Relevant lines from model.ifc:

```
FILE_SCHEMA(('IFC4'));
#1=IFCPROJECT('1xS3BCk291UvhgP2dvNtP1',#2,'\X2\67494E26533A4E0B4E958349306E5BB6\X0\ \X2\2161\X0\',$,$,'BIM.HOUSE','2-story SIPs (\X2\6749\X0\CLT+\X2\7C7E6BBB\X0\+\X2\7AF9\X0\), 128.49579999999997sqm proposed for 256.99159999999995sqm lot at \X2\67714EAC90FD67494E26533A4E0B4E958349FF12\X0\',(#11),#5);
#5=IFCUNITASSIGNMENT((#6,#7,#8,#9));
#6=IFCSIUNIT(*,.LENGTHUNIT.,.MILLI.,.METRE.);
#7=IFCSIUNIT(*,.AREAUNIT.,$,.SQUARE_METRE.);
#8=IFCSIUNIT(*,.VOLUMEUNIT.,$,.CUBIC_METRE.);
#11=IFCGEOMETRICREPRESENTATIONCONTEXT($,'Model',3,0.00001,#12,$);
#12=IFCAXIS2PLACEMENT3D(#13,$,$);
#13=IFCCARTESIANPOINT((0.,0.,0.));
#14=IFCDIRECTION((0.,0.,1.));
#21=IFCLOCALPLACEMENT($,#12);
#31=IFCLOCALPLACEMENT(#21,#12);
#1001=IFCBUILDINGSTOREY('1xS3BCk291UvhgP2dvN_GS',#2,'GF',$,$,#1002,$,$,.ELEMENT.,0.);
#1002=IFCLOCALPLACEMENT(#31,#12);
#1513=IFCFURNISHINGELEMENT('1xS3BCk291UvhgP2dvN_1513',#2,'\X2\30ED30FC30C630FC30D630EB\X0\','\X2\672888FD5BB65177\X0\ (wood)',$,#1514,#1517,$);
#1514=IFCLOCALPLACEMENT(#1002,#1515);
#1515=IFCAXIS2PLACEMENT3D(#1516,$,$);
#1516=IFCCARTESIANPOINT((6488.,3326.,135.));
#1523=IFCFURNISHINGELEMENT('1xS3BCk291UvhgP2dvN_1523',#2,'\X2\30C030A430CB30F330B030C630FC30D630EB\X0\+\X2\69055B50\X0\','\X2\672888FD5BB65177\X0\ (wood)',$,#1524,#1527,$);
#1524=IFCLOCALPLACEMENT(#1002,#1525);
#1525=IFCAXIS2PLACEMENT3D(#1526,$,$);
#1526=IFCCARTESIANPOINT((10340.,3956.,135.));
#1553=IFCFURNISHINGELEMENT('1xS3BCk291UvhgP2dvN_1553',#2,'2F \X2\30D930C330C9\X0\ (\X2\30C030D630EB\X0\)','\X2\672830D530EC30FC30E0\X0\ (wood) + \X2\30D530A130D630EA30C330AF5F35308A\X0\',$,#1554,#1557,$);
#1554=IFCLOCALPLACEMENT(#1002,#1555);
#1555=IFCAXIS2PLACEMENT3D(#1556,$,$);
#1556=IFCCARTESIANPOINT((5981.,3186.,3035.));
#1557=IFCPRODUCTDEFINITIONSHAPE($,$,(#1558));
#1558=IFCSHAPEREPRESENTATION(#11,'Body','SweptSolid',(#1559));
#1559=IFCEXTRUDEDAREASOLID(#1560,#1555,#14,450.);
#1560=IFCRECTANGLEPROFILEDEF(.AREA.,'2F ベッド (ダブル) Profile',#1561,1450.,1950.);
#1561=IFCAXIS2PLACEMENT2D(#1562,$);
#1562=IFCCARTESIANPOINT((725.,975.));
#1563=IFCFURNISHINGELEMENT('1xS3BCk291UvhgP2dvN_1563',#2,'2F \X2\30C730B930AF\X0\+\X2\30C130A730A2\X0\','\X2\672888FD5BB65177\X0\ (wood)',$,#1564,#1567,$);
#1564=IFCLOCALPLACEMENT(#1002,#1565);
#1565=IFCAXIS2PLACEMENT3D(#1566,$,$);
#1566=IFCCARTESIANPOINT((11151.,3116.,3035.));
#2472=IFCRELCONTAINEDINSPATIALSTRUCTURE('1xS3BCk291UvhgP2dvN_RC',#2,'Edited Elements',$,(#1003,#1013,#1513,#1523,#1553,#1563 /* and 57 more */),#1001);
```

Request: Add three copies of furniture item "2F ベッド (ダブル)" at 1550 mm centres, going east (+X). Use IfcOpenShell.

```python
import numpy as np
import ifcopenshell
import ifcopenshell.api.geometry
import ifcopenshell.api.root
import ifcopenshell.util.element
import ifcopenshell.util.placement
import ifcopenshell.util.unit

model = ifcopenshell.open("model.ifc")
unit_scale = ifcopenshell.util.unit.calculate_unit_scale(model)


def reuse_history(source, copy):
    """copy_class also copies each property set's owner history, people and application; keep the originals."""
    for rel in copy.IsDefinedBy:
        if rel.is_a("IfcRelDefinesByProperties") and (history := rel.RelatingPropertyDefinition.OwnerHistory):
            rel.RelatingPropertyDefinition.OwnerHistory = source.OwnerHistory
            ifcopenshell.util.element.remove_deep2(model, history)


source = model.by_id(1553)
base = ifcopenshell.util.placement.get_local_placement(source.ObjectPlacement)
step = np.array([1.0, 0.0, 0.0]) * 1.55 / unit_scale

for i in range(1, 4):
    copy = ifcopenshell.api.root.copy_class(model, product=source)
    copy.Representation = ifcopenshell.util.element.copy_deep(
        model, source.Representation, exclude=["IfcGeometricRepresentationContext", "IfcRepresentationMap"]
    )
    reuse_history(source, copy)
    matrix = base.copy()
    matrix[:3, 3] += i * step
    print("added at", matrix[:3, 3].round(3) + 0.0)
    ifcopenshell.api.geometry.edit_object_placement(model, product=copy, matrix=matrix, is_si=False)

model.write("model_updated.ifc")
```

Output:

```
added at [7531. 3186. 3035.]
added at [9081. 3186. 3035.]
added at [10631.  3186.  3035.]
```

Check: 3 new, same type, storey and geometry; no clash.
